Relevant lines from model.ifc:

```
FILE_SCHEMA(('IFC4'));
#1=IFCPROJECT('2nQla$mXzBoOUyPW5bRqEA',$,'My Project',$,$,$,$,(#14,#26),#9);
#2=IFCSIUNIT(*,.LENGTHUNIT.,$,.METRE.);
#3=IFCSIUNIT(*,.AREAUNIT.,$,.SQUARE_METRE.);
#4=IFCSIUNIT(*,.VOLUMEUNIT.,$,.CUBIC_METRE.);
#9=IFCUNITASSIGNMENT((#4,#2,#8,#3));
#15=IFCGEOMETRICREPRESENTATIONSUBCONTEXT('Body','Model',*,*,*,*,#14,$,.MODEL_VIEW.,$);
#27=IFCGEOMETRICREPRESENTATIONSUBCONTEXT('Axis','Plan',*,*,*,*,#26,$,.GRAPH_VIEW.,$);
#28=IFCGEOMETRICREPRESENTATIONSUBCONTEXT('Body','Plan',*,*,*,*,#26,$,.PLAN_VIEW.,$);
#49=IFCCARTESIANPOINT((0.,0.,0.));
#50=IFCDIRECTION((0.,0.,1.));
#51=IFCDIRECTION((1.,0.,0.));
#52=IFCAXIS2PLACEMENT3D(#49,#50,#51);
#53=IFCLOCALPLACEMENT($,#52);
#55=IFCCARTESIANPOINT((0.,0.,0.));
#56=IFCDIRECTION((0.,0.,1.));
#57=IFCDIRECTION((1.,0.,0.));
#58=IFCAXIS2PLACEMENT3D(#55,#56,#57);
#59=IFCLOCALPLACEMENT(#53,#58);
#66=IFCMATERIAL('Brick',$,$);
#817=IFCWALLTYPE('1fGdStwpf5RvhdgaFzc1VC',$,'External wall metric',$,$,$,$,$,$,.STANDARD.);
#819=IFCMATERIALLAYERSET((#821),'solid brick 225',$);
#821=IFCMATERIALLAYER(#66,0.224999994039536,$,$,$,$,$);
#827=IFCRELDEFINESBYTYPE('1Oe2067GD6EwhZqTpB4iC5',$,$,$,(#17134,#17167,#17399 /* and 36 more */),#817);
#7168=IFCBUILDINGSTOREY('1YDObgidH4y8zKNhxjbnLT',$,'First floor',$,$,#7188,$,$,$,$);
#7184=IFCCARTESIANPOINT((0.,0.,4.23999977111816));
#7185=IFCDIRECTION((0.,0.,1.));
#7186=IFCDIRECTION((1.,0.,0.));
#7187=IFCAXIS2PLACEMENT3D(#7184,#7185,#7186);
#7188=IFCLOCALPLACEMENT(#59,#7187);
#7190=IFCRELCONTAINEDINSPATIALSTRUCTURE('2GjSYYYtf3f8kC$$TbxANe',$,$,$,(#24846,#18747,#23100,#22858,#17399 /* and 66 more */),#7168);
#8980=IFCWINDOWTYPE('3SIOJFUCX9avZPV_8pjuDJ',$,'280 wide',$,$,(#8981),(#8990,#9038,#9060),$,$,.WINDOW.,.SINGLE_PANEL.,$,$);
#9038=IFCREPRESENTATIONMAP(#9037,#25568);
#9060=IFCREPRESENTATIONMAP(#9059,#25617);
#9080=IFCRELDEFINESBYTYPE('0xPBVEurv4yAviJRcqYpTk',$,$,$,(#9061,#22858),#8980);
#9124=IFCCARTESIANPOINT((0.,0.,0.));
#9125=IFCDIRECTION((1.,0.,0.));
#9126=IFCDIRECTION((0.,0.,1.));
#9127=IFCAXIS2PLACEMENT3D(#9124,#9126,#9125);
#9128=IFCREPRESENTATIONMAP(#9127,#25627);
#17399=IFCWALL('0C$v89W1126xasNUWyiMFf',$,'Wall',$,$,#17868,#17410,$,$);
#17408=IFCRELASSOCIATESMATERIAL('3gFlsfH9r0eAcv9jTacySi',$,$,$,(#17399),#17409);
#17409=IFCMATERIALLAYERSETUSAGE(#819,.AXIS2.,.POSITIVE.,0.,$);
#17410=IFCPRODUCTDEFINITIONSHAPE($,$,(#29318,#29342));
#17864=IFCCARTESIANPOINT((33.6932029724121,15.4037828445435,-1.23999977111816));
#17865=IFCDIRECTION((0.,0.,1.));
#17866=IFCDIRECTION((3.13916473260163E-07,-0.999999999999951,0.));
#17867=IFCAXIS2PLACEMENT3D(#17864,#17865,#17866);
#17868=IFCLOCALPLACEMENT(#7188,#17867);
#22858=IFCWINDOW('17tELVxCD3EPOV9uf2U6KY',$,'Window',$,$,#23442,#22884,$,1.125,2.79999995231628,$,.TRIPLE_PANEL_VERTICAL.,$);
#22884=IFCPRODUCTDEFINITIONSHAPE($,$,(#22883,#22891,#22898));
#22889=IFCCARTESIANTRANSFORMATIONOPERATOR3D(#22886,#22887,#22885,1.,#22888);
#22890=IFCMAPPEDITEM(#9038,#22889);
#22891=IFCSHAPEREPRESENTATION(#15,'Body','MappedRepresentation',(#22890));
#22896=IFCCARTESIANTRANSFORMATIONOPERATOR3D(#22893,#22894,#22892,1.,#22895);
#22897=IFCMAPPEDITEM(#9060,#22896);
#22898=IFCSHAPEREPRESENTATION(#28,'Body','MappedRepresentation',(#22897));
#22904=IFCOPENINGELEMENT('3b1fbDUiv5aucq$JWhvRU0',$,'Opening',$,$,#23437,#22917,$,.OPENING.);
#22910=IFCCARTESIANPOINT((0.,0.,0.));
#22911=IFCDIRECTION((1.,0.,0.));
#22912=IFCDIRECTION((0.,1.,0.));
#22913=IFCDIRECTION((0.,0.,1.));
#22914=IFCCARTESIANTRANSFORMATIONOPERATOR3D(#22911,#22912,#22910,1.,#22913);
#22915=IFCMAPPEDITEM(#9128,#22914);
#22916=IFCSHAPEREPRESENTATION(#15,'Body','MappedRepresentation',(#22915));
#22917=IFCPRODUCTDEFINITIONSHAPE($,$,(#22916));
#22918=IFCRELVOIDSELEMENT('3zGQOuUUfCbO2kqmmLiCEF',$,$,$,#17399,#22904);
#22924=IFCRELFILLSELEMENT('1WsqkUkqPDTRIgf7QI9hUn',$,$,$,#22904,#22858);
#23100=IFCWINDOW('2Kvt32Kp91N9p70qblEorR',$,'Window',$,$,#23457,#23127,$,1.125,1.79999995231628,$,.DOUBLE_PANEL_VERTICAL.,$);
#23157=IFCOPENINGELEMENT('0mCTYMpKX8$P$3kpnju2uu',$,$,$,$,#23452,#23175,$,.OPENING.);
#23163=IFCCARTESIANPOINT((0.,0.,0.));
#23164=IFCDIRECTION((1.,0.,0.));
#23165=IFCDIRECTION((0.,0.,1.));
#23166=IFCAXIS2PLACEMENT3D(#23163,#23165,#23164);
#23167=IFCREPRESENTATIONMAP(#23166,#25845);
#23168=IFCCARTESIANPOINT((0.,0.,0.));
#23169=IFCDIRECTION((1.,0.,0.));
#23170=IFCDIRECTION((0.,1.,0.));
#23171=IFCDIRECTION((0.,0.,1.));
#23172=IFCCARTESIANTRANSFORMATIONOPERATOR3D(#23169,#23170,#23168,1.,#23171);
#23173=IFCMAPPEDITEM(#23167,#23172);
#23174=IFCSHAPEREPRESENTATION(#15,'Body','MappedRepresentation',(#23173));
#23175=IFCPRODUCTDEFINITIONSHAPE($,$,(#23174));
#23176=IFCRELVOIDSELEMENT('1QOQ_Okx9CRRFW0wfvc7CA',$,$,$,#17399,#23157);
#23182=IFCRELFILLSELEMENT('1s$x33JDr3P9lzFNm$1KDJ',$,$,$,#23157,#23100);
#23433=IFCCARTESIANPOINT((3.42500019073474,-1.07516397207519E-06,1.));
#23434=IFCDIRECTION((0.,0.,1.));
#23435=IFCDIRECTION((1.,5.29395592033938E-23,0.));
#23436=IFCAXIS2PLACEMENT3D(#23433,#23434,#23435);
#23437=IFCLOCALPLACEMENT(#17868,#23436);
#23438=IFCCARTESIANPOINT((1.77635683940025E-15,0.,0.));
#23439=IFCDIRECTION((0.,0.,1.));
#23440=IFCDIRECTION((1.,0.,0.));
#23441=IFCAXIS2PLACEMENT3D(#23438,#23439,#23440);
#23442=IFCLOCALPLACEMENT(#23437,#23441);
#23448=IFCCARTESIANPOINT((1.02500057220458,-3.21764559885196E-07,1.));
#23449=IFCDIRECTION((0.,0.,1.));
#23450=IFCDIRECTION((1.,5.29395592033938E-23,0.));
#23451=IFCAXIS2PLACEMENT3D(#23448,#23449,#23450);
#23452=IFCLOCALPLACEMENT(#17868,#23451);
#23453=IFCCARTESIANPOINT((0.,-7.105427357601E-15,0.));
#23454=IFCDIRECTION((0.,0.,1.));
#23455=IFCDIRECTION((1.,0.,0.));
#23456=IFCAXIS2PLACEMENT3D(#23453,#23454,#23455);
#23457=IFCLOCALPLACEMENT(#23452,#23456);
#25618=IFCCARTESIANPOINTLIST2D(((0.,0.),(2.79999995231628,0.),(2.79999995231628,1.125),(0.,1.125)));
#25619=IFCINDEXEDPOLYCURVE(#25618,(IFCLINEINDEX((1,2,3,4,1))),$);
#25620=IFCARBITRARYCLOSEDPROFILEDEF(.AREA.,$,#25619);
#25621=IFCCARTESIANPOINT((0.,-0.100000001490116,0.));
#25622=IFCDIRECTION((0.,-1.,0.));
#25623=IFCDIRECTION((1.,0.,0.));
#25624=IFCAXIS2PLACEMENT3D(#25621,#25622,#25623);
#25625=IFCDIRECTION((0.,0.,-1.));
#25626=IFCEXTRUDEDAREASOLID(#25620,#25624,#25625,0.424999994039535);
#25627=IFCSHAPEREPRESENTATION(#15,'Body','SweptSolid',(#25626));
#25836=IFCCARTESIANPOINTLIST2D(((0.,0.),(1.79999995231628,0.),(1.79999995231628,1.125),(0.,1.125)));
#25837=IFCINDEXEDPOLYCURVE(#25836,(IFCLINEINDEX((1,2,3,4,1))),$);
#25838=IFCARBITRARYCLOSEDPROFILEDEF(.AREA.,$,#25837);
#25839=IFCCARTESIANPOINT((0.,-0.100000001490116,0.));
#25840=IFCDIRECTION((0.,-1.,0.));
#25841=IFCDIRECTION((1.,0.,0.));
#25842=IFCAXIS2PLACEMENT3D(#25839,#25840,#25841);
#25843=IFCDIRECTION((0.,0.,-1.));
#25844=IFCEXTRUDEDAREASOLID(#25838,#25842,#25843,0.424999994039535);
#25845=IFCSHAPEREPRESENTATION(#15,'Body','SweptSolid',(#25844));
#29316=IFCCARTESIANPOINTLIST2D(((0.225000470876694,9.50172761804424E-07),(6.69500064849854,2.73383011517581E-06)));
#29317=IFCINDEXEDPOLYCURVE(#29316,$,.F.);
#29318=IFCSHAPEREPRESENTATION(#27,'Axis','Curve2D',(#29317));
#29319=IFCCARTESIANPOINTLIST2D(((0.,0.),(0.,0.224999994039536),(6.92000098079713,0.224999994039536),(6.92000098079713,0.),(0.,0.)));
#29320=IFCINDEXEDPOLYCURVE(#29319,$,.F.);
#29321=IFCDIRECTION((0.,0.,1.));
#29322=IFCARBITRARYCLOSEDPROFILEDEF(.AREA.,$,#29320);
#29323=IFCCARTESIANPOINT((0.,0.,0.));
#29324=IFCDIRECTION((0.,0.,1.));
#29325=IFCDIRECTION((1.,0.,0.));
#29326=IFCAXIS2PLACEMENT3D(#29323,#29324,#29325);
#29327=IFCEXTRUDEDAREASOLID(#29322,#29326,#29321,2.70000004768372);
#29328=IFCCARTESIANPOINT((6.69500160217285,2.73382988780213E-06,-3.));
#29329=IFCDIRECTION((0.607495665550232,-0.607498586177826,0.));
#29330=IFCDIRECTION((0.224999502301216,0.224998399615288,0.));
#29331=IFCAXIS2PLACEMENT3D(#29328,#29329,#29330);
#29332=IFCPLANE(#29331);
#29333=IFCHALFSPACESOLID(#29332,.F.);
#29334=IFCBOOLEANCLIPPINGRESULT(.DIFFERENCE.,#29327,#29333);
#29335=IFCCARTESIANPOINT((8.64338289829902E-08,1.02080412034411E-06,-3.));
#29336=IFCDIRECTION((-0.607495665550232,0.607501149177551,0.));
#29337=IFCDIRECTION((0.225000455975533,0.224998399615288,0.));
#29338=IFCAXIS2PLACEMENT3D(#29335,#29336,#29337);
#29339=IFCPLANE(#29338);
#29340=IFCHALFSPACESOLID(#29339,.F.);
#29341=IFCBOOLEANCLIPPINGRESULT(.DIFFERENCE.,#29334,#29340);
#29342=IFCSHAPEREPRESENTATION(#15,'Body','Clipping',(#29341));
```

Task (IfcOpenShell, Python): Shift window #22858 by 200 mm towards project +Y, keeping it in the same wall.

```python
import ifcopenshell
import ifcopenshell.api.geometry
import ifcopenshell.util.placement

model = ifcopenshell.open("model.ifc")

window = model.by_guid("17tELVxCD3EPOV9uf2U6KY")
opening = window.FillsVoids[0].RelatingOpeningElement
wall = opening.VoidsElements[0].RelatingBuildingElement

wall_matrix = ifcopenshell.util.placement.get_local_placement(wall.ObjectPlacement)
shift = wall_matrix[:3, 0] * -0.2
before = ifcopenshell.util.placement.get_local_placement(window.ObjectPlacement)[:3, 3].copy()

# The window is placed relative to its opening, so it follows when the opening moves.
matrix = ifcopenshell.util.placement.get_local_placement(opening.ObjectPlacement)
matrix[:3, 3] += shift
ifcopenshell.api.geometry.edit_object_placement(
    model, product=opening, matrix=matrix, is_si=False, should_transform_children=True
)

after = ifcopenshell.util.placement.get_local_placement(window.ObjectPlacement)[:3, 3]
print("window moved by", (after - before).round(3) + 0.0)

model.write("model_edited.ifc")
```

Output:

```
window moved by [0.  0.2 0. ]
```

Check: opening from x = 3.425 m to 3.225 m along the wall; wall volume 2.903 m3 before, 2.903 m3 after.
